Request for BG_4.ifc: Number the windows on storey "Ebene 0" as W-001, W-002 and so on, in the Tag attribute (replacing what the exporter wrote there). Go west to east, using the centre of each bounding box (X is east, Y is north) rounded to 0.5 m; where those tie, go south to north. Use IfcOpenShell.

First a look at what the model holds.

```python
import ifcopenshell
import ifcopenshell.util.element
import ifcopenshell.util.placement

model = ifcopenshell.open("BG_4.ifc")
print(model.schema)
storey = next(s for s in model.by_type("IfcBuildingStorey") if s.Name == "Ebene 0")
windows = [e for e in ifcopenshell.util.element.get_decomposition(storey) if e.is_a("IfcWindow")]
for e in sorted(windows, key=lambda e: e.id()):
    origin = ifcopenshell.util.placement.get_local_placement(e.ObjectPlacement)[:3, 3]
    print(e.id(), e.Tag, e.Name, origin.round(2) + 0.0, sep=" | ")
```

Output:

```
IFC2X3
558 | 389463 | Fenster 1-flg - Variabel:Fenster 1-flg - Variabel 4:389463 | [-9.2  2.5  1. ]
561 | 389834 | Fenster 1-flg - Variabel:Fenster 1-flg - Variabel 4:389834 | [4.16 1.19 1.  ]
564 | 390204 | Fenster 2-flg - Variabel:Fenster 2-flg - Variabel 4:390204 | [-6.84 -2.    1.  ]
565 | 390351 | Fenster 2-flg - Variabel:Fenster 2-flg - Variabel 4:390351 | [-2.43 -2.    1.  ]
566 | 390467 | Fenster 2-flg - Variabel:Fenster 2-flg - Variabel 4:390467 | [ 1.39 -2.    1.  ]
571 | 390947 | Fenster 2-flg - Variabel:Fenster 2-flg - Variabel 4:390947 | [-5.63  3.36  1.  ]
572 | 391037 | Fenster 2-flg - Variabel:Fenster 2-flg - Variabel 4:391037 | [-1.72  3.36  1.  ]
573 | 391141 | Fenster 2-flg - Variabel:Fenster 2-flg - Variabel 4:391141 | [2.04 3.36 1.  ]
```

```python
import ifcopenshell
import ifcopenshell.geom
import ifcopenshell.util.element
import ifcopenshell.util.shape

model = ifcopenshell.open("BG_4.ifc")
settings = ifcopenshell.geom.settings()
settings.set("use-world-coords", True)


def centre(element):
    shape = ifcopenshell.geom.create_shape(settings, element)
    return ifcopenshell.util.shape.get_bbox_centroid(shape.geometry)


storey = next(s for s in model.by_type("IfcBuildingStorey") if s.Name == "Ebene 0")
windows = [e for e in ifcopenshell.util.element.get_decomposition(storey) if e.is_a("IfcWindow")]

# Insertion points can sit at a corner or the storey origin, so sort by the geometry (in metres).
centres = {e: centre(e) for e in windows}
windows.sort(key=lambda e: (round(centres[e][0] / 0.5), centres[e][1]))

for i, e in enumerate(windows, start=1):
    number = f"W-0{i:02d}"
    e.Tag = number
    print(e.id(), number)

model.write("BG_4_rev.ifc")
```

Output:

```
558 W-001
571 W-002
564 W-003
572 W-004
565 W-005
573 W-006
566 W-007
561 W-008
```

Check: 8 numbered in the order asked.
